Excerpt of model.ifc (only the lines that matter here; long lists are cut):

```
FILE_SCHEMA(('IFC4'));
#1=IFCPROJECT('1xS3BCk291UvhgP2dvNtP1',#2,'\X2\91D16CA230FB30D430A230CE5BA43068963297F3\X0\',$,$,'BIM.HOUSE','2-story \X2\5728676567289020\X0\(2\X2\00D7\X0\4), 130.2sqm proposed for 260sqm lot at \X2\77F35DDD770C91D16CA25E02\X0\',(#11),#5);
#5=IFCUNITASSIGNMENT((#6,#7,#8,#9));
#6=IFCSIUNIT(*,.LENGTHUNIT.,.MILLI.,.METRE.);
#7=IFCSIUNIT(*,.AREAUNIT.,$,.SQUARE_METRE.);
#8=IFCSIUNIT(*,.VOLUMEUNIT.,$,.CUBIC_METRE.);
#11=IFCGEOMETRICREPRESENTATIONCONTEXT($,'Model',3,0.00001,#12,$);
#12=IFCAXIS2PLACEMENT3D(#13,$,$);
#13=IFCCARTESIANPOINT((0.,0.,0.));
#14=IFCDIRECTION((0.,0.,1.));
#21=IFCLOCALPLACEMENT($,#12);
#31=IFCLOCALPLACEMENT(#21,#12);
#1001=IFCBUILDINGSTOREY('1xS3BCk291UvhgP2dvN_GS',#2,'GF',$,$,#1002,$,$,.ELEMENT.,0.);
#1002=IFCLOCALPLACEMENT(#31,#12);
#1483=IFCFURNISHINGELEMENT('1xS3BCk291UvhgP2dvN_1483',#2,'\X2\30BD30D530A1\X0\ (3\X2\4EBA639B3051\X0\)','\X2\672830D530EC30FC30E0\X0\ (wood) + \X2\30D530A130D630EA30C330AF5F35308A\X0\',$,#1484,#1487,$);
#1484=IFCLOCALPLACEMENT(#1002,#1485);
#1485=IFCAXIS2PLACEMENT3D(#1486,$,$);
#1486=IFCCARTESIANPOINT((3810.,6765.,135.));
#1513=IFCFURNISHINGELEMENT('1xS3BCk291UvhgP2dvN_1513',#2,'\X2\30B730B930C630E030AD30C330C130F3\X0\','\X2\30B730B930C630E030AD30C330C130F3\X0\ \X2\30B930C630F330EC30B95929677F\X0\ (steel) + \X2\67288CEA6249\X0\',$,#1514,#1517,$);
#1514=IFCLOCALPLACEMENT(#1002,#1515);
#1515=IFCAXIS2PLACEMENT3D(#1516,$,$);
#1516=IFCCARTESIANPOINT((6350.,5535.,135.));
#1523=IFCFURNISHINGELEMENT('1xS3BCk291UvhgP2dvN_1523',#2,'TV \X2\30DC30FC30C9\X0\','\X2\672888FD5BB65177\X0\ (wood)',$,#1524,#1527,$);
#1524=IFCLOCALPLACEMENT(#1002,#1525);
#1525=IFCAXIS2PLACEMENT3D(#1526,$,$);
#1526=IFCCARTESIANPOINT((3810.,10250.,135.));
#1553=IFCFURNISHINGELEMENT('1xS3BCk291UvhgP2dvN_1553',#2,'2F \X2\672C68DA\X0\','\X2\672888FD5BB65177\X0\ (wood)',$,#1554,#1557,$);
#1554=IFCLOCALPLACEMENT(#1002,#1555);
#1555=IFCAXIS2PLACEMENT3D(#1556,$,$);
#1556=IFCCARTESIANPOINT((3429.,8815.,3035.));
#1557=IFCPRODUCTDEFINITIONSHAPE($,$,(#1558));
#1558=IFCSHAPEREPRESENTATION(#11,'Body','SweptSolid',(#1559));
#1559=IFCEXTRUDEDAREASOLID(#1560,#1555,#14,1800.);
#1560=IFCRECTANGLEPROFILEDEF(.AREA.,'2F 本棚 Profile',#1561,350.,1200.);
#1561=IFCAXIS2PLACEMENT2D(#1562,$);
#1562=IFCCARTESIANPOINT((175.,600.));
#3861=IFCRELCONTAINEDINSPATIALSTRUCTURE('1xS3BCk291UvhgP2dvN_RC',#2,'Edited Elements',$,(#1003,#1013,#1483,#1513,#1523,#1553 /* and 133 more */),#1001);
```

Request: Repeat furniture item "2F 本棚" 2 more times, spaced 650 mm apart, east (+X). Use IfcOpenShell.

```python
import numpy as np
import ifcopenshell
import ifcopenshell.api.geometry
import ifcopenshell.api.root
import ifcopenshell.util.element
import ifcopenshell.util.placement
import ifcopenshell.util.unit

model = ifcopenshell.open("model.ifc")
unit_scale = ifcopenshell.util.unit.calculate_unit_scale(model)


def reuse_history(source, copy):
    """copy_class also copies each property set's owner history, people and application; keep the originals."""
    for rel in copy.IsDefinedBy:
        if rel.is_a("IfcRelDefinesByProperties") and (history := rel.RelatingPropertyDefinition.OwnerHistory):
            rel.RelatingPropertyDefinition.OwnerHistory = source.OwnerHistory
            ifcopenshell.util.element.remove_deep2(model, history)


source = model.by_guid("1xS3BCk291UvhgP2dvN_1553")
base = ifcopenshell.util.placement.get_local_placement(source.ObjectPlacement)
step = np.array([1.0, 0.0, 0.0]) * 0.65 / unit_scale

for i in range(1, 3):
    copy = ifcopenshell.api.root.copy_class(model, product=source)
    copy.Representation = ifcopenshell.util.element.copy_deep(
        model, source.Representation, exclude=["IfcGeometricRepresentationContext", "IfcRepresentationMap"]
    )
    reuse_history(source, copy)
    matrix = base.copy()
    matrix[:3, 3] += i * step
    print("added at", matrix[:3, 3].round(3) + 0.0)
    ifcopenshell.api.geometry.edit_object_placement(model, product=copy, matrix=matrix, is_si=False)

model.write("model-out.ifc")
```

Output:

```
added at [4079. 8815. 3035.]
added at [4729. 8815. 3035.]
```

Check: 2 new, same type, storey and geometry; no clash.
